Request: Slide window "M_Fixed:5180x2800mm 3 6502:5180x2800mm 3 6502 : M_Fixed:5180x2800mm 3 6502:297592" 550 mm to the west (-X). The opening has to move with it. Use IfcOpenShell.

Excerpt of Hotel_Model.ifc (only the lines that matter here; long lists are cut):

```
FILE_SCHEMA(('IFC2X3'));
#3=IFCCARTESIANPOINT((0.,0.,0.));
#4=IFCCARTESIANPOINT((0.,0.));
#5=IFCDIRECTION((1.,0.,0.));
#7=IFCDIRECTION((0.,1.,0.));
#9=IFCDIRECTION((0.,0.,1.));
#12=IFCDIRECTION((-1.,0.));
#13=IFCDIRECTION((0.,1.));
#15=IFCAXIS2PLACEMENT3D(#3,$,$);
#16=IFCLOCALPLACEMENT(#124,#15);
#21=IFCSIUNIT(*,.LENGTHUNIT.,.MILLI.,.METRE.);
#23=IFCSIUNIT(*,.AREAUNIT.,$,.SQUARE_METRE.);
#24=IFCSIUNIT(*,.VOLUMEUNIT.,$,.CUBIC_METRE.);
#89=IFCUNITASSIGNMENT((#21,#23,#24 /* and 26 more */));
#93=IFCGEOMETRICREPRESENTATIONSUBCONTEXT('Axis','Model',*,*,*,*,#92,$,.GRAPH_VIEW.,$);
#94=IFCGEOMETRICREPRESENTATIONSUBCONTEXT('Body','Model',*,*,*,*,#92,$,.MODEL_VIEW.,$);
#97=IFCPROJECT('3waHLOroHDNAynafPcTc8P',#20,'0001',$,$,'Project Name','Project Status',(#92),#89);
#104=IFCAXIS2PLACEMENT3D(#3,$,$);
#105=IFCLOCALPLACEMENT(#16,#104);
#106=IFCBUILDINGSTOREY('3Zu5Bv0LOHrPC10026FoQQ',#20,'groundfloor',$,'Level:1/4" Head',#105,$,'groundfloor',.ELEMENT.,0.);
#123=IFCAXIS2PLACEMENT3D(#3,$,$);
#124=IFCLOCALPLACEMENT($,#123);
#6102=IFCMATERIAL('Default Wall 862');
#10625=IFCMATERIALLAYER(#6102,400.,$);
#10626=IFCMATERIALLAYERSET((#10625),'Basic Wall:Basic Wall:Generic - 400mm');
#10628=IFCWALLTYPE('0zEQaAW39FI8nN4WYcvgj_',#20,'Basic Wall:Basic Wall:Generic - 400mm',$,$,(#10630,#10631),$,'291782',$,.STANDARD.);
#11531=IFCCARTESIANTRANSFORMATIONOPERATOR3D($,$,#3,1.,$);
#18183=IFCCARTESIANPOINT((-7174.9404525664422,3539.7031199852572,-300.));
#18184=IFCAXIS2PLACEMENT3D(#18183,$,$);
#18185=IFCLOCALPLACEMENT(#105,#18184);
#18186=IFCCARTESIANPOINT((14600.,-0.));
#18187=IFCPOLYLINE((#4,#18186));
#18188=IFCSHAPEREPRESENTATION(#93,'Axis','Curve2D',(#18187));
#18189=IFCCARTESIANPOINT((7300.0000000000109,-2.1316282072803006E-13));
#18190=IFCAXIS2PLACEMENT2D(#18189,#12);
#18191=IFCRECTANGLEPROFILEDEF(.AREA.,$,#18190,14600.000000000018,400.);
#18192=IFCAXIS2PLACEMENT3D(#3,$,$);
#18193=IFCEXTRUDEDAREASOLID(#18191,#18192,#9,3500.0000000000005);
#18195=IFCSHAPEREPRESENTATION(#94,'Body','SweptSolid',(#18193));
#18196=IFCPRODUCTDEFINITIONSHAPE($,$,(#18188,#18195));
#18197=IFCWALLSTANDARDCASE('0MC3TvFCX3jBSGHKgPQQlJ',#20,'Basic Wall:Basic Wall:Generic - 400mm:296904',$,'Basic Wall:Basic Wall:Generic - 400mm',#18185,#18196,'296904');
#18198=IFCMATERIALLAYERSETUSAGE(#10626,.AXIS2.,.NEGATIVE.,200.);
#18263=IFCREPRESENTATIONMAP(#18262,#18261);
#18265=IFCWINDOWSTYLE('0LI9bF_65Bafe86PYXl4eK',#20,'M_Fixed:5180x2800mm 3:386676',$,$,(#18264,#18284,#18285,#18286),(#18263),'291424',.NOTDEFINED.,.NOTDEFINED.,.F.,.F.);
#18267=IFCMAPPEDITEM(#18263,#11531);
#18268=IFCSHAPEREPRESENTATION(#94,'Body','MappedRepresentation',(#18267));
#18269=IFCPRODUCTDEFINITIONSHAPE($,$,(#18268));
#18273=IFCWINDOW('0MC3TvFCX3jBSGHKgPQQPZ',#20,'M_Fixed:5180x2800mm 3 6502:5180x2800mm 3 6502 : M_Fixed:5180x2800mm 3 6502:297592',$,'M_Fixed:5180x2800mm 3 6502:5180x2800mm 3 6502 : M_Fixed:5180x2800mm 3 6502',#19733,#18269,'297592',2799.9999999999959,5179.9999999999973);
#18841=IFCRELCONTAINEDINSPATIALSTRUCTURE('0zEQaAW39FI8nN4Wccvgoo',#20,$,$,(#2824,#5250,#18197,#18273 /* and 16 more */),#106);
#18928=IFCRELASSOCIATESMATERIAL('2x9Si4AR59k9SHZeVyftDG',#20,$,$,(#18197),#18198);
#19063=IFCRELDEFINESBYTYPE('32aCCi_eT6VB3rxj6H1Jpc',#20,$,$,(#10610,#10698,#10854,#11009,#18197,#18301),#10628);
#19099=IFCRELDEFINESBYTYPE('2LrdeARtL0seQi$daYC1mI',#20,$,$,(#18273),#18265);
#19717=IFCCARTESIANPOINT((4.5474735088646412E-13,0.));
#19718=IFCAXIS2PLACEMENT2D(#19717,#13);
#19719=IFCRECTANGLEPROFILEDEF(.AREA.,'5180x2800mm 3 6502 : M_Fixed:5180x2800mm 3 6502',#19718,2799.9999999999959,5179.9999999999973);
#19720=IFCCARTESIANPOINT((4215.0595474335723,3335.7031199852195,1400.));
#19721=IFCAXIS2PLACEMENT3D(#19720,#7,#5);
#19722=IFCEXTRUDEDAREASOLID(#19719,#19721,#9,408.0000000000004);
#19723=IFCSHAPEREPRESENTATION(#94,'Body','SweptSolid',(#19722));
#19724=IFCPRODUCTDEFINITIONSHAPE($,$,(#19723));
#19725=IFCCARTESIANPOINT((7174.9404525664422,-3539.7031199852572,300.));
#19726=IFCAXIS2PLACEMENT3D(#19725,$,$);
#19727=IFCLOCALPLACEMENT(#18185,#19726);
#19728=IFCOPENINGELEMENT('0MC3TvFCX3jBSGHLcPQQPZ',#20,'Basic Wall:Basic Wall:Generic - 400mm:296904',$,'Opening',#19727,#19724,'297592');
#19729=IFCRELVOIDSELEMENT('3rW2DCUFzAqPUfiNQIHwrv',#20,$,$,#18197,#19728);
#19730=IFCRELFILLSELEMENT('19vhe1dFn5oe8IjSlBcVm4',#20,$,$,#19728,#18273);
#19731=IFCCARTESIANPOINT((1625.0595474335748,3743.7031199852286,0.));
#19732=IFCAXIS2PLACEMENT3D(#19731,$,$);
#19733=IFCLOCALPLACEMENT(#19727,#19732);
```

```python
import ifcopenshell
import ifcopenshell.api.geometry
import ifcopenshell.util.placement
import ifcopenshell.util.unit

model = ifcopenshell.open("Hotel_Model.ifc")
unit_scale = ifcopenshell.util.unit.calculate_unit_scale(model)

window = model.by_guid("0MC3TvFCX3jBSGHKgPQQPZ")
opening = window.FillsVoids[0].RelatingOpeningElement
wall = opening.VoidsElements[0].RelatingBuildingElement

wall_matrix = ifcopenshell.util.placement.get_local_placement(wall.ObjectPlacement)
shift = wall_matrix[:3, 0] * -0.55 / unit_scale
before = ifcopenshell.util.placement.get_local_placement(window.ObjectPlacement)[:3, 3].copy()

# The window is placed relative to its opening, so it follows when the opening moves.
matrix = ifcopenshell.util.placement.get_local_placement(opening.ObjectPlacement)
matrix[:3, 3] += shift
ifcopenshell.api.geometry.edit_object_placement(
    model, product=opening, matrix=matrix, is_si=False, should_transform_children=True
)

after = ifcopenshell.util.placement.get_local_placement(window.ObjectPlacement)[:3, 3]
print("window moved by", (after - before).round(3) + 0.0)

model.write("Hotel_Model_edited.ifc")
```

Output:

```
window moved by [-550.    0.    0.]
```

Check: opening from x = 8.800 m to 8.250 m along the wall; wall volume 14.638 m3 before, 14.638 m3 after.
